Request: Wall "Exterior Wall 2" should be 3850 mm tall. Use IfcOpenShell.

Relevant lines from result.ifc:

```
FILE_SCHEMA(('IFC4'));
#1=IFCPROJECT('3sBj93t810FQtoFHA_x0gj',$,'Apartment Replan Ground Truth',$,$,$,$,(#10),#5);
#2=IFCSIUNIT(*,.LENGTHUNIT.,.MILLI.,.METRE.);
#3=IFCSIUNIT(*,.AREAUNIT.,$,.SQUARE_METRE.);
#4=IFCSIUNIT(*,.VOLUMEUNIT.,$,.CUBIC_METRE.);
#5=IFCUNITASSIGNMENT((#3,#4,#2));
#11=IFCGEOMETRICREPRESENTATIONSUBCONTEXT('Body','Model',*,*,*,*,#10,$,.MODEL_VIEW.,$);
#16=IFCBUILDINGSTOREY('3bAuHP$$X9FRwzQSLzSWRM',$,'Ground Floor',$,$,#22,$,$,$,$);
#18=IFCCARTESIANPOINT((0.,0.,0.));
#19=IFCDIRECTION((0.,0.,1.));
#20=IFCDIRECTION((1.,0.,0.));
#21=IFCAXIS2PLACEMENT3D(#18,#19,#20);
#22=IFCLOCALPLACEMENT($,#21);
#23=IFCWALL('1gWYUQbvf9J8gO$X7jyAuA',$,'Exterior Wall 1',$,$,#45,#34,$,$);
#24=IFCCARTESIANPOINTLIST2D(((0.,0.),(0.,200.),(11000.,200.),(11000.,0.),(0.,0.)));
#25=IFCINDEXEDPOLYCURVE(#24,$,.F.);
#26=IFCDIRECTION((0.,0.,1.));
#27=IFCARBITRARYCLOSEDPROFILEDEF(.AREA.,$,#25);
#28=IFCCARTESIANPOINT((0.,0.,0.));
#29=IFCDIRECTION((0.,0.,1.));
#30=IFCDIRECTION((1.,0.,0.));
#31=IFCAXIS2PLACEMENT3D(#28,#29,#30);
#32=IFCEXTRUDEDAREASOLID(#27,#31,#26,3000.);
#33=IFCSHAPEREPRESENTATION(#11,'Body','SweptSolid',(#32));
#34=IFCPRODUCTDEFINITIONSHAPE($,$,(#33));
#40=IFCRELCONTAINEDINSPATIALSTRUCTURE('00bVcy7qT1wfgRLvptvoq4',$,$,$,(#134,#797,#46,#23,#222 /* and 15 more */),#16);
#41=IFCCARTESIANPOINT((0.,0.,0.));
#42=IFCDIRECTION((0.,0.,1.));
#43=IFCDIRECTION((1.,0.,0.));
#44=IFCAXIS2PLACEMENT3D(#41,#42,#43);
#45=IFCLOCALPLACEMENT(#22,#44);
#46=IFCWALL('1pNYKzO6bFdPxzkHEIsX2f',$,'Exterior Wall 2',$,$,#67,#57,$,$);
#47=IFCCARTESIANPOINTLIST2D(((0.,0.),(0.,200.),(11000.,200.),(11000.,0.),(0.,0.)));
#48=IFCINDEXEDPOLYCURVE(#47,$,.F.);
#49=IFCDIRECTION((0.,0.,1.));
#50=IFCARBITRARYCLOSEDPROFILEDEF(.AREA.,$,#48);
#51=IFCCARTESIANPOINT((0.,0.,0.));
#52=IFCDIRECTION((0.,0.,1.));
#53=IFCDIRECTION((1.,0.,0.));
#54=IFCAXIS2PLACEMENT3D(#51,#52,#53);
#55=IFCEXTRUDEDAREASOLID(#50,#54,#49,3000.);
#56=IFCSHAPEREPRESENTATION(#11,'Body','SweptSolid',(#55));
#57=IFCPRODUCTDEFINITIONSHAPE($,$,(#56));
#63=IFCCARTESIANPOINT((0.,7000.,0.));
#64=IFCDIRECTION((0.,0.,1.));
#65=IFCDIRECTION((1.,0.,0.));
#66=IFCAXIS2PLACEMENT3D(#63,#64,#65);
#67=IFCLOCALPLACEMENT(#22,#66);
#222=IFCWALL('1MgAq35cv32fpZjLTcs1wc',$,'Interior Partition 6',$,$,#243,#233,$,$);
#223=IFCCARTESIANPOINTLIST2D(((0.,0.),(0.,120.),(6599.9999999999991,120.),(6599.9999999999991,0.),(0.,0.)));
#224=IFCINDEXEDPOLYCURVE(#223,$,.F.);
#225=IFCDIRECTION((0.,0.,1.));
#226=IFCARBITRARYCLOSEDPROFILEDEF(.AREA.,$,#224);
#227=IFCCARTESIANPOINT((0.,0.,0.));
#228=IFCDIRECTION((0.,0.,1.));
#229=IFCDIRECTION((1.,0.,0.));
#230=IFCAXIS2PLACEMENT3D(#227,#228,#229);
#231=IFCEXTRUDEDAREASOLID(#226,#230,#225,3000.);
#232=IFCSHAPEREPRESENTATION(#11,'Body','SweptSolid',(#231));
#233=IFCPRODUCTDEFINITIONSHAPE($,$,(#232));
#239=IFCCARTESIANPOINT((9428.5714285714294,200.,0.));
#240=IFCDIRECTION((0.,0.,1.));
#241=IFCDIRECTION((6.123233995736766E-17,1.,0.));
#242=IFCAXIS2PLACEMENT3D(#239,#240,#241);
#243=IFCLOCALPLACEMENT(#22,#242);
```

```python
import ifcopenshell
import ifcopenshell.geom
import ifcopenshell.util.representation
import ifcopenshell.util.shape
import ifcopenshell.util.unit

model = ifcopenshell.open("result.ifc")
unit_scale = ifcopenshell.util.unit.calculate_unit_scale(model)
settings = ifcopenshell.geom.settings()


def volume(element):
    """Net volume in cubic metres, openings subtracted."""
    shape = ifcopenshell.geom.create_shape(settings, element)
    return ifcopenshell.util.shape.get_volume(shape.geometry)


wall = model.by_guid("1pNYKzO6bFdPxzkHEIsX2f")
before = volume(wall)

body = ifcopenshell.util.representation.get_representation(wall, "Model", "Body")
solid = body.Items[0]
old_height = solid.Depth
solid.Depth = 3.85 / unit_scale
after = volume(wall)

print(f"height {old_height:g} -> {solid.Depth:g}, volume {before:.3f} -> {after:.3f} m3")

model.write("result_edited.ifc")
```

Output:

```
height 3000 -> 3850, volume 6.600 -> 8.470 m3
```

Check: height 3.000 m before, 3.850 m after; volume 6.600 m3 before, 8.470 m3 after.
